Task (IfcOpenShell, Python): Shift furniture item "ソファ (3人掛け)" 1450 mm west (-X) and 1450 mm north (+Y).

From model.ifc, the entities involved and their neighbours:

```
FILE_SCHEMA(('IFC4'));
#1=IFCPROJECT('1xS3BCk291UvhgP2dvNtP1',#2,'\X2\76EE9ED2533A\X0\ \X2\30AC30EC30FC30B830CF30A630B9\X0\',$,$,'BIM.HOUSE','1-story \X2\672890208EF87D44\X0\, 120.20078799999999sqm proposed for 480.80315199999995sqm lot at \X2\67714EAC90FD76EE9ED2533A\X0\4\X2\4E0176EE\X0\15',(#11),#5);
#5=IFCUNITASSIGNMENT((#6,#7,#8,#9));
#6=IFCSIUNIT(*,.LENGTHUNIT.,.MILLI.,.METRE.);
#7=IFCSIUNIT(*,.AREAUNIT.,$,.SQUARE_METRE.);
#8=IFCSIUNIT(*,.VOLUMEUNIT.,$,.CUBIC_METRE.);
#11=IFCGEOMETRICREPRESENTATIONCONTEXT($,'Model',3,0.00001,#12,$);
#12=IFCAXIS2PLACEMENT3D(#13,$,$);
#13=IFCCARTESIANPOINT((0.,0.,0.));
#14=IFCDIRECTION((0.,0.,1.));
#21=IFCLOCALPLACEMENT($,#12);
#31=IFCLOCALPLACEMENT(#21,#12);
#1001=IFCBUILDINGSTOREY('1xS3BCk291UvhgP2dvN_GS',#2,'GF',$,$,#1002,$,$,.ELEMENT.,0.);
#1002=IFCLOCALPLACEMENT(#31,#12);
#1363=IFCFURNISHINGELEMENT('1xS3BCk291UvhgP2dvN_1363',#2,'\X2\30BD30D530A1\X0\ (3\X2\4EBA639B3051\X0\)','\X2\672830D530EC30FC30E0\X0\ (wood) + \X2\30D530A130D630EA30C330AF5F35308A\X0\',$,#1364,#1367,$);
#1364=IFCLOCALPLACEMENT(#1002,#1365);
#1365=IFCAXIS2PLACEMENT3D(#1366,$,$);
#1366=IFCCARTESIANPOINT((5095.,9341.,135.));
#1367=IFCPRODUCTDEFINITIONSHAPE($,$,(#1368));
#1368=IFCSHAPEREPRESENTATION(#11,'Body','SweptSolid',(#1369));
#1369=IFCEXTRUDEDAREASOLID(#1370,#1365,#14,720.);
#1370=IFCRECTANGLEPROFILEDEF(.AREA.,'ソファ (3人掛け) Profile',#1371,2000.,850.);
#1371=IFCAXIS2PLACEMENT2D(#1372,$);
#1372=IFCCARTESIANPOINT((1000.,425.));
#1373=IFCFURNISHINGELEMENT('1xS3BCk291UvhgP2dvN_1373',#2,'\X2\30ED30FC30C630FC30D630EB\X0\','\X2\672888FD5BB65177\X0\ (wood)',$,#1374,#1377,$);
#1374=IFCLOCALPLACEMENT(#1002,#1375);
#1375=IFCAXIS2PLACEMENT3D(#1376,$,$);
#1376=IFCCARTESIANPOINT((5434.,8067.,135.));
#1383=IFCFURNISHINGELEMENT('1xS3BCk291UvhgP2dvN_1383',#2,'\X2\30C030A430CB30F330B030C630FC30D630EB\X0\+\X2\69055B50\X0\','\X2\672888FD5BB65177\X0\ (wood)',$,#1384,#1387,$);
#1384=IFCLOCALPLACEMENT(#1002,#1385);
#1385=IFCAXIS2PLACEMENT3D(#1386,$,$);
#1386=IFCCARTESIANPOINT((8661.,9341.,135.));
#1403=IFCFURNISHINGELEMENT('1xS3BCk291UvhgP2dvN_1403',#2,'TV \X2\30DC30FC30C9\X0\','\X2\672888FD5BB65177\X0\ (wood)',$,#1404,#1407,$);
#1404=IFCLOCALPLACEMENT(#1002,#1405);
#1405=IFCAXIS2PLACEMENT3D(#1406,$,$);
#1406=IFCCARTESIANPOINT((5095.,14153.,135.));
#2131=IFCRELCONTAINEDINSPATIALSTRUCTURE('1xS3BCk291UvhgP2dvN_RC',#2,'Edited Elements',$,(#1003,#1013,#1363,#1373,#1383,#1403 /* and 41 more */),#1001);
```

```python
import ifcopenshell
import ifcopenshell.api.geometry
import ifcopenshell.util.placement
import ifcopenshell.util.unit

model = ifcopenshell.open("model.ifc")
unit_scale = ifcopenshell.util.unit.calculate_unit_scale(model)

item = model.by_guid("1xS3BCk291UvhgP2dvN_1363")
matrix = ifcopenshell.util.placement.get_local_placement(item.ObjectPlacement)
matrix[0, 3] -= 1.45 / unit_scale
matrix[1, 3] += 1.45 / unit_scale
ifcopenshell.api.geometry.edit_object_placement(model, product=item, matrix=matrix, is_si=False)

print(ifcopenshell.util.placement.get_local_placement(item.ObjectPlacement).round(3) + 0.0)

model.write("model_updated.ifc")
```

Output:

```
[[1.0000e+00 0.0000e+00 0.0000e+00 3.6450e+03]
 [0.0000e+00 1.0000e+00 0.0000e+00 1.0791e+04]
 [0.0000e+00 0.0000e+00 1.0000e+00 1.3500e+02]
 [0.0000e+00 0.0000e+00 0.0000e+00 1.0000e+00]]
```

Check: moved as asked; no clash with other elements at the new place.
